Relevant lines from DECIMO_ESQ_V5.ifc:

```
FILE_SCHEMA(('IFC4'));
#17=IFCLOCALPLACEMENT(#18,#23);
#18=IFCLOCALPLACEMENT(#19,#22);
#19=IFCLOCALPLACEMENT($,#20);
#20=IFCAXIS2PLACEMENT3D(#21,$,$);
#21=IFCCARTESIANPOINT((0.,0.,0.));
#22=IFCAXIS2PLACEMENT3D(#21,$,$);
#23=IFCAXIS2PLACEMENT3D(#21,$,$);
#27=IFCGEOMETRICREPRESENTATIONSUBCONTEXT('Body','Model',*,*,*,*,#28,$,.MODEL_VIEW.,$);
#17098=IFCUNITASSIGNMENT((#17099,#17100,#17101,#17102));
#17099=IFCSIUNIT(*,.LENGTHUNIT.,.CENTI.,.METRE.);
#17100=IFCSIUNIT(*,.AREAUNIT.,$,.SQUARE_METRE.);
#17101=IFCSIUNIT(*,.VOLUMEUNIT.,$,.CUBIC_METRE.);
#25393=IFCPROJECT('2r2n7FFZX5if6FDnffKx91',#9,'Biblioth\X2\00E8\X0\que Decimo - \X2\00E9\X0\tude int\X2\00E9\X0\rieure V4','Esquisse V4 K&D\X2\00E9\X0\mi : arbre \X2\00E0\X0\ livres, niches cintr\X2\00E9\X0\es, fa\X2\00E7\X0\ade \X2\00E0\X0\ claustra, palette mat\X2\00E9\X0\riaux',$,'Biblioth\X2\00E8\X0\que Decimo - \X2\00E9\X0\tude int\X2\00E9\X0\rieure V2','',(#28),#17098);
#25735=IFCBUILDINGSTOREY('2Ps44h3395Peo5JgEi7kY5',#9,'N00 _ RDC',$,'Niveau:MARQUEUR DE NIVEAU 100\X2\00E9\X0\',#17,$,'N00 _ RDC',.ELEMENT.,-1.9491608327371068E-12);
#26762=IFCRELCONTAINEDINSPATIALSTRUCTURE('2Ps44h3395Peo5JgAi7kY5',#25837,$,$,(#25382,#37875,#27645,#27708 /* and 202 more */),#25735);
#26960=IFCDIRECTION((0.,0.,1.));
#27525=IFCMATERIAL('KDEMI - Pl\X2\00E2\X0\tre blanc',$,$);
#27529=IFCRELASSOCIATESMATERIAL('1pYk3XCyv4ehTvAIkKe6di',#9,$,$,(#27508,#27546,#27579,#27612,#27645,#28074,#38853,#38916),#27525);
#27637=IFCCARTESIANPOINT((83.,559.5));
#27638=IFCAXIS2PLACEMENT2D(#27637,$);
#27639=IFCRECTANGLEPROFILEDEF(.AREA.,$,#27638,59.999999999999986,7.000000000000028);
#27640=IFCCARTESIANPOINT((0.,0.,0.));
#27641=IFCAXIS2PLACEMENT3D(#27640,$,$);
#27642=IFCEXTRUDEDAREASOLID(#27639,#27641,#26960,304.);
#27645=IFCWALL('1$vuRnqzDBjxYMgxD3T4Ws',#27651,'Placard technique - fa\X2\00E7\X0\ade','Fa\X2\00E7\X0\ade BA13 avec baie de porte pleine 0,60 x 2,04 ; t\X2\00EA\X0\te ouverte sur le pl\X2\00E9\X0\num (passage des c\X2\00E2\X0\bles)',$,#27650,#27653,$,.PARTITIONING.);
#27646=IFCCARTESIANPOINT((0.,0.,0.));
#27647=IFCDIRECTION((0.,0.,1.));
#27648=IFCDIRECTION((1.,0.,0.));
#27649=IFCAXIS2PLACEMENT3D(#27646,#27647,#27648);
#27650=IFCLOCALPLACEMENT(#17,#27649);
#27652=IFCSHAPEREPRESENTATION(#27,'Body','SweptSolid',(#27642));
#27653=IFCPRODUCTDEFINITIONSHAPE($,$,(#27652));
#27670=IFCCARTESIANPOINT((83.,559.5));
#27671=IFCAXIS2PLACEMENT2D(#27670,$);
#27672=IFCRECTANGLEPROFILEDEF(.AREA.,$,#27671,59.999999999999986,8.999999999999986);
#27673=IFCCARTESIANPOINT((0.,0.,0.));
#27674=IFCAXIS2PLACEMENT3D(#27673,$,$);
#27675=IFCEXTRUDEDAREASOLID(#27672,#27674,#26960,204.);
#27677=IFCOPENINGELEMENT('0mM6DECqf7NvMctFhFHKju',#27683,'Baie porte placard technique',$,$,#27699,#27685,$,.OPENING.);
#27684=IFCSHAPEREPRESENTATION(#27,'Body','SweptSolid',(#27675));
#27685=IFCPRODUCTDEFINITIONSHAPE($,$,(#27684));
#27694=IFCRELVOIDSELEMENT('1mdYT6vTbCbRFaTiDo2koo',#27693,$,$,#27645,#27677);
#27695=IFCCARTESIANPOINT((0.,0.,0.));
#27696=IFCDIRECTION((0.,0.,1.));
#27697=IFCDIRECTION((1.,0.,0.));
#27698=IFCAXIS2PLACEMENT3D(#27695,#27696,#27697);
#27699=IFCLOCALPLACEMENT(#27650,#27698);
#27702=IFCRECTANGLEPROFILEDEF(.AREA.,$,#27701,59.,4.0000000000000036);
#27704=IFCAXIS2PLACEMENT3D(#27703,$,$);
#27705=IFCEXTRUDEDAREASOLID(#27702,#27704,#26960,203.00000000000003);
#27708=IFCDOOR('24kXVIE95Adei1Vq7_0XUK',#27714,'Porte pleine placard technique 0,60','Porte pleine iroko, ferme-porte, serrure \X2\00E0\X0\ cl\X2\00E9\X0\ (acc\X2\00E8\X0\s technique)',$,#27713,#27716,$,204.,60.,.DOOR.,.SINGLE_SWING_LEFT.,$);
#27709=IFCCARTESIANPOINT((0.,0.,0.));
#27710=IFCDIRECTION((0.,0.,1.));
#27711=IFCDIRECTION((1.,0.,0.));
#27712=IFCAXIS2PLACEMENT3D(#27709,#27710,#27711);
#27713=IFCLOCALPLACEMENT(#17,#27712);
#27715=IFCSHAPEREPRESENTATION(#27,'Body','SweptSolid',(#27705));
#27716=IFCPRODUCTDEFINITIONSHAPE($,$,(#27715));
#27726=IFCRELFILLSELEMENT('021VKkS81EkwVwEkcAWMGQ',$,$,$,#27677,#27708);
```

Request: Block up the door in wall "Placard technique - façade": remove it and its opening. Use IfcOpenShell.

```python
import ifcopenshell
import ifcopenshell.api.feature
import ifcopenshell.api.root
import ifcopenshell.geom
import ifcopenshell.util.shape

model = ifcopenshell.open("DECIMO_ESQ_V5.ifc")
settings = ifcopenshell.geom.settings()


def volume(element):
    """Net volume in cubic metres, openings subtracted."""
    shape = ifcopenshell.geom.create_shape(settings, element)
    return ifcopenshell.util.shape.get_volume(shape.geometry)


door = model.by_id(27708)
opening = door.FillsVoids[0].RelatingOpeningElement
wall = opening.VoidsElements[0].RelatingBuildingElement
before = volume(wall)

ifcopenshell.api.root.remove_product(model, product=door)
ifcopenshell.api.feature.remove_feature(model, feature=opening)

after = volume(wall)

print(f"wall volume {before:.3f} -> {after:.3f} m3")

model.write("DECIMO_ESQ_V5_rev.ifc")
```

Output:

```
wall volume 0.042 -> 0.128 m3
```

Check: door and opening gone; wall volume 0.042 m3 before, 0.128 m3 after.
